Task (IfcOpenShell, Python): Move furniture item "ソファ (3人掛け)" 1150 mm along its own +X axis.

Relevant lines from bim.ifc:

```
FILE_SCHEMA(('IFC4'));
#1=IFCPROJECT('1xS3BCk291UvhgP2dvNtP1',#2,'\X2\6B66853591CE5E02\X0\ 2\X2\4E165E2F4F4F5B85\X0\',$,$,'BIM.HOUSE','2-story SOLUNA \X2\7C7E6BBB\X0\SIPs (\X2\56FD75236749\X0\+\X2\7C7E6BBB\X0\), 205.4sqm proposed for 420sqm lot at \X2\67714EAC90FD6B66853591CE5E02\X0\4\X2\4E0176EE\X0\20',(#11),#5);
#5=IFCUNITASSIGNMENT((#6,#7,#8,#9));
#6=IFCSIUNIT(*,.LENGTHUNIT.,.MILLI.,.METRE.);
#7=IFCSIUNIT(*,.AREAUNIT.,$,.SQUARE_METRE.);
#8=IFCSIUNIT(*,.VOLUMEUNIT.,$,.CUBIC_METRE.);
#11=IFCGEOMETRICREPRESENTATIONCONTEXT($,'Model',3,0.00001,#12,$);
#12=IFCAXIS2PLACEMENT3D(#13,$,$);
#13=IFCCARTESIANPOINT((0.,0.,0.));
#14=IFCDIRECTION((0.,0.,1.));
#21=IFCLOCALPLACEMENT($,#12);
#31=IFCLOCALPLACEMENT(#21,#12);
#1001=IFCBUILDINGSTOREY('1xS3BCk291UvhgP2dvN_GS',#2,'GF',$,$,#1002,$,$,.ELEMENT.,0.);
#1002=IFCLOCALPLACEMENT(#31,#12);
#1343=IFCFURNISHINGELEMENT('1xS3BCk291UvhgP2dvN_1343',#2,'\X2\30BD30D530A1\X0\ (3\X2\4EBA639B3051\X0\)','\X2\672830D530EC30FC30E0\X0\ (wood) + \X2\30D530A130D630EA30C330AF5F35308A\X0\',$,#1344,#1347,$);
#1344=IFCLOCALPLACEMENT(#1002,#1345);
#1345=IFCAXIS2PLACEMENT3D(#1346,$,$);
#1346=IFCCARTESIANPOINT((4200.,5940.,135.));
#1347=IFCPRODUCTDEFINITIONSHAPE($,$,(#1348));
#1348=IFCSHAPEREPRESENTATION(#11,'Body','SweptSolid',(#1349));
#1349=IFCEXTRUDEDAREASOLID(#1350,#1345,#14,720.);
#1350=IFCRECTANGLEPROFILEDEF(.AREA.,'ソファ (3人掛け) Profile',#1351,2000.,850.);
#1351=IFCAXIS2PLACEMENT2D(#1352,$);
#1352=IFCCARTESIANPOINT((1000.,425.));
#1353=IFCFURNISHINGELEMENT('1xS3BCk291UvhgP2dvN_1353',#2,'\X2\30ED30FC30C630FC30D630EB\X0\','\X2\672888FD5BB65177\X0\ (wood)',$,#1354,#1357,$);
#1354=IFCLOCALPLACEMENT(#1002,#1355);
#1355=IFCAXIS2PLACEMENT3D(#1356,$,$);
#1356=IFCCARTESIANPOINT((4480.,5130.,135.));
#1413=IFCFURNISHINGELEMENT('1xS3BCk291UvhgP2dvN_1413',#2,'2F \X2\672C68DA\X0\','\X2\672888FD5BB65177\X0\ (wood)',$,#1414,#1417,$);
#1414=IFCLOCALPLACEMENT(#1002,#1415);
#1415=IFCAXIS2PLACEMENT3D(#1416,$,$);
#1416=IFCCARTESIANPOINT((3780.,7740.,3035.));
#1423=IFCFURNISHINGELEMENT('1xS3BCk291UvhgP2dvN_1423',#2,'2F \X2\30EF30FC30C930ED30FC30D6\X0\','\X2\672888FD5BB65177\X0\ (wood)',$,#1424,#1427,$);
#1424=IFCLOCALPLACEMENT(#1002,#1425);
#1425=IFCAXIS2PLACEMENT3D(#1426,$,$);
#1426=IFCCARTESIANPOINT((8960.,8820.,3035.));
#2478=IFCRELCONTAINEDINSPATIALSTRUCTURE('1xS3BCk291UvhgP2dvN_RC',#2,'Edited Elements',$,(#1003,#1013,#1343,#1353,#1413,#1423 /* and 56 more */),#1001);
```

```python
import ifcopenshell
import ifcopenshell.api.geometry
import ifcopenshell.util.placement
import ifcopenshell.util.unit

model = ifcopenshell.open("bim.ifc")
unit_scale = ifcopenshell.util.unit.calculate_unit_scale(model)

item = model.by_id(1343)
matrix = ifcopenshell.util.placement.get_local_placement(item.ObjectPlacement)
matrix[:3, 3] += matrix[:3, 0] * 1.15 / unit_scale
ifcopenshell.api.geometry.edit_object_placement(model, product=item, matrix=matrix, is_si=False)

print(ifcopenshell.util.placement.get_local_placement(item.ObjectPlacement).round(3) + 0.0)

model.write("bim_updated.ifc")
```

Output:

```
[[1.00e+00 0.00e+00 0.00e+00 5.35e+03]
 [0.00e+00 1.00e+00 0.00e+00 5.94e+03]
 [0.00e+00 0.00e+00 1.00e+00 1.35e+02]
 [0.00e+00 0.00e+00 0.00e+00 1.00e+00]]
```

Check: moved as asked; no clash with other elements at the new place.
